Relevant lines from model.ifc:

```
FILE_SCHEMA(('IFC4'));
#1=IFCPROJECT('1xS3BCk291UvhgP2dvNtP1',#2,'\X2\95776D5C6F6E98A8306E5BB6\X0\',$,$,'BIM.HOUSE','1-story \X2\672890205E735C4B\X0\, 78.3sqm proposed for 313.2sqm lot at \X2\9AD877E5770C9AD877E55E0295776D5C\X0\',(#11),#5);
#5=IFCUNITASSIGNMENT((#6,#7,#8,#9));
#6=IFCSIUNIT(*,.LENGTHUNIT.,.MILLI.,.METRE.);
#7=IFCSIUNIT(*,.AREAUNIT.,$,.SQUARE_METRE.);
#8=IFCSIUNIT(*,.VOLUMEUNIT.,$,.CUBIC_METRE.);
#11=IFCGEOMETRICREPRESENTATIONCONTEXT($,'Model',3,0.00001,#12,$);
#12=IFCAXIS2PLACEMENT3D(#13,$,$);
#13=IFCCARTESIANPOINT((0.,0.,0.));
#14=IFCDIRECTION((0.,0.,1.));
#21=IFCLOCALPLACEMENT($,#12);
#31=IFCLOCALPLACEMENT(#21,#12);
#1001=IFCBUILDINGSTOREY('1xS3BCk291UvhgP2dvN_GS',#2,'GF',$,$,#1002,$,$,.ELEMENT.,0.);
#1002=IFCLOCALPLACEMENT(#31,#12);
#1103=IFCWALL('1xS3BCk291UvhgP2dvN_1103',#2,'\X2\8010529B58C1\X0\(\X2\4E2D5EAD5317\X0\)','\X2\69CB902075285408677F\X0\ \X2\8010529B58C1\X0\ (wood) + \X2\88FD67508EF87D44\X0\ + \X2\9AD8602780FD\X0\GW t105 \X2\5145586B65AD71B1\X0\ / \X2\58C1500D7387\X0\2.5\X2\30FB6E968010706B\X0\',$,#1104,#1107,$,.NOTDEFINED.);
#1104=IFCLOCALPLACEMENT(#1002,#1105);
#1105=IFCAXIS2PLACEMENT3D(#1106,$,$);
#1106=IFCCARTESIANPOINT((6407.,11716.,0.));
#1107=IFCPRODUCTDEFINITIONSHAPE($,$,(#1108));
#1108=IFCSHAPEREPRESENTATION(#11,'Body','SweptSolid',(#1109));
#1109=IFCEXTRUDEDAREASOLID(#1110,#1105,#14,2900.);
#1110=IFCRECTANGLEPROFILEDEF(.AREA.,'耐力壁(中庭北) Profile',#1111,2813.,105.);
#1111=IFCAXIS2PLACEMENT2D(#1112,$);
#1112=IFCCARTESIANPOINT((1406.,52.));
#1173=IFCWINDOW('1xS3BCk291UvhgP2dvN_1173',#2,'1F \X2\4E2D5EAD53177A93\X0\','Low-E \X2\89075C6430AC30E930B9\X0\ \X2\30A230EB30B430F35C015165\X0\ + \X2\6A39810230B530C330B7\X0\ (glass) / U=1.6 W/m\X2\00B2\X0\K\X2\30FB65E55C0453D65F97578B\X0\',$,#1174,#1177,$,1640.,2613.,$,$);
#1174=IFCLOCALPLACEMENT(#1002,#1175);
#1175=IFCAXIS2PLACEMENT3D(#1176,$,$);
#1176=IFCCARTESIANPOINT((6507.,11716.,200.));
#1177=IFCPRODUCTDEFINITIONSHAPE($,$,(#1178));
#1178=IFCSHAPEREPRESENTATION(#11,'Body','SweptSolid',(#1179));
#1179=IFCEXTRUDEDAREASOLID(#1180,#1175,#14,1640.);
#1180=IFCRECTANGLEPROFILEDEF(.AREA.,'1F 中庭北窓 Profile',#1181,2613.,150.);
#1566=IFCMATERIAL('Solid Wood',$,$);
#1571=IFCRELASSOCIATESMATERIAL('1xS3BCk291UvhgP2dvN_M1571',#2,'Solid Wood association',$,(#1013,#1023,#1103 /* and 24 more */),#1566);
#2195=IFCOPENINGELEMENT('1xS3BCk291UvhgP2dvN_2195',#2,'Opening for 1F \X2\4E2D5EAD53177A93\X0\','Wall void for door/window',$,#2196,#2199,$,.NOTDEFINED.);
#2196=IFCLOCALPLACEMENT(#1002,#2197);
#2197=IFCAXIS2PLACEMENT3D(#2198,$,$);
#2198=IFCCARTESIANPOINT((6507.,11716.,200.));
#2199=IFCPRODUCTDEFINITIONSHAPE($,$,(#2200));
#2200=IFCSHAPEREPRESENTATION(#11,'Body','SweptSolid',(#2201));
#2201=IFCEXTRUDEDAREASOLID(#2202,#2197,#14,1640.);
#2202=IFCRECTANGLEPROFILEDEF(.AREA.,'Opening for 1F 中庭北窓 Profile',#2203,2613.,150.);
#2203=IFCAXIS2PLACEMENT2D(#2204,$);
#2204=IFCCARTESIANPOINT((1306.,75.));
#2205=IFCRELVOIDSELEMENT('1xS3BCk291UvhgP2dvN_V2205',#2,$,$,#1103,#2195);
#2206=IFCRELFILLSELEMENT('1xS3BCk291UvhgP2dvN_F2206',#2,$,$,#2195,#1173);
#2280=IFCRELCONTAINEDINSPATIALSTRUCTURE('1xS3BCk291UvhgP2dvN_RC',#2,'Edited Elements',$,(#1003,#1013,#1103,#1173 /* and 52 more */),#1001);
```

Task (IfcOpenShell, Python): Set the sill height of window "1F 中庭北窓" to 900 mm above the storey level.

```python
import numpy as np
import ifcopenshell
import ifcopenshell.api.geometry
import ifcopenshell.geom
import ifcopenshell.util.element
import ifcopenshell.util.placement
import ifcopenshell.util.shape
import ifcopenshell.util.unit

model = ifcopenshell.open("model.ifc")
unit_scale = ifcopenshell.util.unit.calculate_unit_scale(model)

window = model.by_id(1173)
opening = window.FillsVoids[0].RelatingOpeningElement
storey = ifcopenshell.util.element.get_container(window, ifc_class="IfcBuildingStorey")
level = ifcopenshell.util.placement.get_local_placement(storey.ObjectPlacement)[2, 3]

# The opening's origin need not be at the sill, so measure its lowest point.
shape = ifcopenshell.geom.create_shape(ifcopenshell.geom.settings(), opening)
bottom = ifcopenshell.util.shape.get_shape_bottom_elevation(shape, shape.geometry) / unit_scale
dz = level + 900.0 - bottom

shift = np.array([0.0, 0.0, dz])
# The window is not placed relative to its opening, so move both.
for product in (opening, window):
    matrix = ifcopenshell.util.placement.get_local_placement(product.ObjectPlacement)
    matrix[:3, 3] += shift
    ifcopenshell.api.geometry.edit_object_placement(model, product=product, matrix=matrix, is_si=False)

print(f"moved by {dz * unit_scale:+.3f} m")

model.write("model-out.ifc")
```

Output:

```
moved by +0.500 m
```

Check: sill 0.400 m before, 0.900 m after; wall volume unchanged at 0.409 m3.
